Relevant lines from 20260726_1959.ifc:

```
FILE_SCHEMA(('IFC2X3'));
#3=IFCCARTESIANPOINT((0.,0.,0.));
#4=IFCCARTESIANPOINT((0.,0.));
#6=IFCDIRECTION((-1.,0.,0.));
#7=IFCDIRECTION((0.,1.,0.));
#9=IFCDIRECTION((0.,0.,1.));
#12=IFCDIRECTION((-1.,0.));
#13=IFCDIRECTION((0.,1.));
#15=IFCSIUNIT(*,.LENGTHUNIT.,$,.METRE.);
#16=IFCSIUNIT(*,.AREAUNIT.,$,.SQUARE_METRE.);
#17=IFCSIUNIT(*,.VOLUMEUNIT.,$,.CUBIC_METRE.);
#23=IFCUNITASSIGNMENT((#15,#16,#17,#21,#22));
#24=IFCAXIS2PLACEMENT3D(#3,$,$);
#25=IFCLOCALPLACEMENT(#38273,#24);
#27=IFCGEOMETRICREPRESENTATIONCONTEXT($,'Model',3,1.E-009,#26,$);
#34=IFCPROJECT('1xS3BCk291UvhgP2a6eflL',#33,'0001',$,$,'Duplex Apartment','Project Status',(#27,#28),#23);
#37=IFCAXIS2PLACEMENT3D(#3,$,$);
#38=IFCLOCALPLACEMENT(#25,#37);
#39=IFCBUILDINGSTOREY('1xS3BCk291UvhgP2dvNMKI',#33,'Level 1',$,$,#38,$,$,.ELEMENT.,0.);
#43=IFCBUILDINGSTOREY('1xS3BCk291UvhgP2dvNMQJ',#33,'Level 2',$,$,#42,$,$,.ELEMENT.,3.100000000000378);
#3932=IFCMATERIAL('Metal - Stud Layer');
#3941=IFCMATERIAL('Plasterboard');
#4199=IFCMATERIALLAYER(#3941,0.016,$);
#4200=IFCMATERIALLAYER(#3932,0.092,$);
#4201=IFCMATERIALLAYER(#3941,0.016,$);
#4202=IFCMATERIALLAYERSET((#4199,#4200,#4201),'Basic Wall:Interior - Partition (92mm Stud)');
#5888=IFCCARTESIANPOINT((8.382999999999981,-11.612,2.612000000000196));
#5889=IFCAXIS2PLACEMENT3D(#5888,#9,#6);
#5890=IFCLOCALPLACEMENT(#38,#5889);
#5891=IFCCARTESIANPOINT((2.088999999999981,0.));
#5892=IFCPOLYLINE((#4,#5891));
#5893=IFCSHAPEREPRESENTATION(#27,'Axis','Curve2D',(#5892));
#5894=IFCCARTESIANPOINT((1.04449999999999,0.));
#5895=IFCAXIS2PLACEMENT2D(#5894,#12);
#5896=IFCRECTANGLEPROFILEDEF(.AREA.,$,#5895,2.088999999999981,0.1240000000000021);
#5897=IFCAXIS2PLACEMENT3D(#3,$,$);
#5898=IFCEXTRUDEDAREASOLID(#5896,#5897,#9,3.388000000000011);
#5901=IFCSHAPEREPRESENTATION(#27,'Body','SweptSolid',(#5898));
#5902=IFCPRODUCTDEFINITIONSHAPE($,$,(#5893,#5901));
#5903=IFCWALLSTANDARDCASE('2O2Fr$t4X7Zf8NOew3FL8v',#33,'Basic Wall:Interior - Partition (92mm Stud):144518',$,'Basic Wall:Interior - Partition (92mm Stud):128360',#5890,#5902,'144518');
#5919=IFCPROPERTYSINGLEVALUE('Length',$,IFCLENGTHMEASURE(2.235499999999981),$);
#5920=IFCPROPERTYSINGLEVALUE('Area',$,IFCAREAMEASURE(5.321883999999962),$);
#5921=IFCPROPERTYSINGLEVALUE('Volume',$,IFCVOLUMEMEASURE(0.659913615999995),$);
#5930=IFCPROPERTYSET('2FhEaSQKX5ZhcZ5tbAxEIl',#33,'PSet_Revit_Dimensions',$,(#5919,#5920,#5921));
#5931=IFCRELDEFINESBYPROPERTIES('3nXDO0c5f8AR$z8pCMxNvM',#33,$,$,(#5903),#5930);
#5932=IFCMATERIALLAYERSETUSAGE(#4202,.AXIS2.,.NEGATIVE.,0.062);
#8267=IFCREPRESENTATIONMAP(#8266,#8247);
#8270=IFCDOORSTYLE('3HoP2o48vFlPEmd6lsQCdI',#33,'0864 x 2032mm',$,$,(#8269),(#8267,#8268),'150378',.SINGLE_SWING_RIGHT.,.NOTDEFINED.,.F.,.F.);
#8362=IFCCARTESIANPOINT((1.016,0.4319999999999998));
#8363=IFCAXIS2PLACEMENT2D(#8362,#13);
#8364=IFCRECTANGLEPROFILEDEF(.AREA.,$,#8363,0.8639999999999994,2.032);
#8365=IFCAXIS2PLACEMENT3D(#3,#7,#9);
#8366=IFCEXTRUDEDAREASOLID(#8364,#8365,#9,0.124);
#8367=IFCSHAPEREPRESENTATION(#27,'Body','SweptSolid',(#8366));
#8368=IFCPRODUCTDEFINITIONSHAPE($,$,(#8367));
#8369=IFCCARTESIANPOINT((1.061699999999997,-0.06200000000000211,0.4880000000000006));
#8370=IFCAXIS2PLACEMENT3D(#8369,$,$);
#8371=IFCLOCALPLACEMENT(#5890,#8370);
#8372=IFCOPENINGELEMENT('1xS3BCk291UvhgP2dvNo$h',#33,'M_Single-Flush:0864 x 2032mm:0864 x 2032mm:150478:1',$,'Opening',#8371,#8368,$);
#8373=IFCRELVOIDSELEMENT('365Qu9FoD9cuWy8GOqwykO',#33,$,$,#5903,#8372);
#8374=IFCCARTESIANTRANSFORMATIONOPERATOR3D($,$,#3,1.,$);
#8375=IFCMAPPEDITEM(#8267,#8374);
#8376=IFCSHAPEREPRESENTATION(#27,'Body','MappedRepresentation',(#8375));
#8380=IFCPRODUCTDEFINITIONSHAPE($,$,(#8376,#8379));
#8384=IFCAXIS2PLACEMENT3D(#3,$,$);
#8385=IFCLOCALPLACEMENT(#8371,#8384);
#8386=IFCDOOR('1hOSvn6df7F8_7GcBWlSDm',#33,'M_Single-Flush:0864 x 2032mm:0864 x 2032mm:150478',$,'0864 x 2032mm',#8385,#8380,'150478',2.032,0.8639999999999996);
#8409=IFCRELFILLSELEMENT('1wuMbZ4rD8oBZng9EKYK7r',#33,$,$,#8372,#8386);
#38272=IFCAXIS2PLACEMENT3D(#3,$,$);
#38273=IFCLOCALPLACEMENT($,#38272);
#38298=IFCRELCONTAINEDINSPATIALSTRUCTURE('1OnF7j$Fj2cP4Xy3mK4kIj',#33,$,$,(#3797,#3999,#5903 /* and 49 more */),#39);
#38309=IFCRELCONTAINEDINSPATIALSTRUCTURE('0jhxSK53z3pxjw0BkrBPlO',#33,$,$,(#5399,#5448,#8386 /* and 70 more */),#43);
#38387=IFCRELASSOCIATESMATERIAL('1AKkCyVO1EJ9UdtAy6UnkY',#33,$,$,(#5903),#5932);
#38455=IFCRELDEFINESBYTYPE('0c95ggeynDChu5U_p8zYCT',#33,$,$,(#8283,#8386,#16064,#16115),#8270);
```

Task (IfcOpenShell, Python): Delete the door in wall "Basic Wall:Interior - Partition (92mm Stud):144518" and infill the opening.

```python
import ifcopenshell
import ifcopenshell.api.feature
import ifcopenshell.api.pset
import ifcopenshell.api.root
import ifcopenshell.geom
import ifcopenshell.util.element
import ifcopenshell.util.shape
import ifcopenshell.util.unit

model = ifcopenshell.open("20260726_1959.ifc")
area_scale = ifcopenshell.util.unit.calculate_unit_scale(model, "AREAUNIT")
volume_scale = ifcopenshell.util.unit.calculate_unit_scale(model, "VOLUMEUNIT")
settings = ifcopenshell.geom.settings()


def volume(element):
    """Net volume in cubic metres, openings subtracted."""
    shape = ifcopenshell.geom.create_shape(settings, element)
    return ifcopenshell.util.shape.get_volume(shape.geometry)


door = model.by_id(8386)
opening = door.FillsVoids[0].RelatingOpeningElement
wall = opening.VoidsElements[0].RelatingBuildingElement
before = volume(wall)

ifcopenshell.api.root.remove_product(model, product=door)
ifcopenshell.api.feature.remove_feature(model, feature=opening)

after = volume(wall)
thickness = 0.124  # wall thickness in metres

# Update the wall's stored quantities.
pset = model.by_id(ifcopenshell.util.element.get_pset(wall, "PSet_Revit_Dimensions", should_inherit=False)["id"])
ifcopenshell.api.pset.edit_pset(model, pset=pset, properties={
    "Area": model.create_entity("IfcAreaMeasure", after / thickness / area_scale),
    "Volume": model.create_entity("IfcVolumeMeasure", after / volume_scale),
})

print(f"wall volume {before:.3f} -> {after:.3f} m3")

model.write("20260726_1959_updated.ifc")
```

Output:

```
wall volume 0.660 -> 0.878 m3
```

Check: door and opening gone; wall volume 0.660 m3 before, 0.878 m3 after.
